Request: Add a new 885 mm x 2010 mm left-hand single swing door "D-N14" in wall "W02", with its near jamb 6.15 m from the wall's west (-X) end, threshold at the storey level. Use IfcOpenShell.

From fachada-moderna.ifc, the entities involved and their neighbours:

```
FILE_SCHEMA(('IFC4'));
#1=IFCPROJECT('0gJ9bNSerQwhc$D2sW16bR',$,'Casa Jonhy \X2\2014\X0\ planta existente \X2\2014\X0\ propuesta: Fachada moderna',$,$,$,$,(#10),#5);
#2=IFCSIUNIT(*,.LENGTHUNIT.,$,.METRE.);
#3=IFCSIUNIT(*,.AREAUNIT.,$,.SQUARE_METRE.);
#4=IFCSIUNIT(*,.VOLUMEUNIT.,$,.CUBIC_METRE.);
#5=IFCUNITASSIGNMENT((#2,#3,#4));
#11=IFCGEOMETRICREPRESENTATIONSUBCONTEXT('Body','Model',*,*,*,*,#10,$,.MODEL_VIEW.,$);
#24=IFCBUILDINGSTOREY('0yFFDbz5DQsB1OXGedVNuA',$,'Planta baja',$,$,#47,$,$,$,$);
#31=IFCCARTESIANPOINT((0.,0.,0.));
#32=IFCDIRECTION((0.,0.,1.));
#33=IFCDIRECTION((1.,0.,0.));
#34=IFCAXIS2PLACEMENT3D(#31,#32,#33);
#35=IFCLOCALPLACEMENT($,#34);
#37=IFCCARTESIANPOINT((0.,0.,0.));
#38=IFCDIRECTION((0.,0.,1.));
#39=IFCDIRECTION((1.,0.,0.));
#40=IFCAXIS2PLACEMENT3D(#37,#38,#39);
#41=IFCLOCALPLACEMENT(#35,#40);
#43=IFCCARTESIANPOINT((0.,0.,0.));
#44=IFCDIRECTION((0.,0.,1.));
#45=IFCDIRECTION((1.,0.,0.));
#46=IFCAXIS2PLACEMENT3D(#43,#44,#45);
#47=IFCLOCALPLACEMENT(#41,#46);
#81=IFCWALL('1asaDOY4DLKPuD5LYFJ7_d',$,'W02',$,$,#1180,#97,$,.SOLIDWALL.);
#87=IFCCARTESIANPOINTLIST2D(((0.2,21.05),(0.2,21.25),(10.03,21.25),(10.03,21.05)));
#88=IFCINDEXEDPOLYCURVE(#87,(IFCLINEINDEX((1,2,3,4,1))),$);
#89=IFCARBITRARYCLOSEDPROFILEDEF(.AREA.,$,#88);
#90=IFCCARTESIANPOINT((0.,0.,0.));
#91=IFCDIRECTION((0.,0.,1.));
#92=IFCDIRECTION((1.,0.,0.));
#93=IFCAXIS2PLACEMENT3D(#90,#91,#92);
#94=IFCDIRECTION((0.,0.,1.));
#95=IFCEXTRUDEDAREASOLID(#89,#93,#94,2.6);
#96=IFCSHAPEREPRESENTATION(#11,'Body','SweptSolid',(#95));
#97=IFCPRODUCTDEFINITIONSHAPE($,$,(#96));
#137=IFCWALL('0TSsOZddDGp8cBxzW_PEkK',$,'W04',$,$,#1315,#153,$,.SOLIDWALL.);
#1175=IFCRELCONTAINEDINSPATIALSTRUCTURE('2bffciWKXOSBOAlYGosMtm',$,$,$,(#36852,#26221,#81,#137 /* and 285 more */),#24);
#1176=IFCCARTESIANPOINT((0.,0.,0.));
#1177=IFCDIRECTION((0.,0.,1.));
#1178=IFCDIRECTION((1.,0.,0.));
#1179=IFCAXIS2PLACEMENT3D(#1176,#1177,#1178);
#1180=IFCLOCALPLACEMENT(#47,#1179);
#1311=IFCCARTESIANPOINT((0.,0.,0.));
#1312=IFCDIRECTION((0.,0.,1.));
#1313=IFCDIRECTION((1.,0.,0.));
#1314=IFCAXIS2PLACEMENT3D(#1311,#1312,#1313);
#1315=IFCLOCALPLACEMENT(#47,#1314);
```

```python
import numpy as np
import ifcopenshell
import ifcopenshell.api.feature
import ifcopenshell.api.geometry
import ifcopenshell.api.root
import ifcopenshell.api.spatial
import ifcopenshell.geom
import ifcopenshell.util.element
import ifcopenshell.util.placement
import ifcopenshell.util.representation
import ifcopenshell.util.shape
import ifcopenshell.util.unit

model = ifcopenshell.open("fachada-moderna.ifc")
unit_scale = ifcopenshell.util.unit.calculate_unit_scale(model)
settings = ifcopenshell.geom.settings()


def volume(element):
    """Net volume in cubic metres, openings subtracted."""
    shape = ifcopenshell.geom.create_shape(settings, element)
    return ifcopenshell.util.shape.get_volume(shape.geometry)


wall = model.by_guid("1asaDOY4DLKPuD5LYFJ7_d")
storey = ifcopenshell.util.element.get_container(wall, ifc_class="IfcBuildingStorey")
context = ifcopenshell.util.representation.get_context(model, "Model", "Body", "MODEL_VIEW")
before = volume(wall)

width, height, from_end, sill = 0.885, 2.01, 6.15, 0.0  # metres

# The wall runs along its own X axis, and the end named is its -X end.
wall_shape = ifcopenshell.geom.create_shape(settings, wall)
x, y, z = ifcopenshell.util.shape.get_vertices(wall_shape.geometry).T
start = x.min() + from_end
face, thickness = float(y.min()), float(y.max() - y.min())
wall_matrix = ifcopenshell.util.placement.get_local_placement(wall.ObjectPlacement)
level = ifcopenshell.util.placement.get_local_placement(storey.ObjectPlacement)[2, 3]


def in_wall(x, y):
    """Placement at x, y metres in the wall's axes, at sill height."""
    matrix = wall_matrix.copy()
    matrix[:, 3] = wall_matrix @ np.array([x / unit_scale, y / unit_scale, 0.0, 1.0])
    matrix[2, 3] = level + sill / unit_scale
    return matrix


# Opening: a box that overshoots both wall faces by 50 mm.
opening = ifcopenshell.api.root.create_entity(model, ifc_class="IfcOpeningElement", predefined_type="OPENING")
box = ifcopenshell.api.geometry.add_wall_representation(
    model, context=context, length=width, height=height, thickness=thickness + 0.1
)
ifcopenshell.api.geometry.assign_representation(model, product=opening, representation=box)
ifcopenshell.api.geometry.edit_object_placement(model, product=opening, matrix=in_wall(start, face - 0.05), is_si=False)
ifcopenshell.api.feature.add_feature(model, feature=opening, element=wall)

door = ifcopenshell.api.root.create_entity(model, ifc_class="IfcDoor", name="D-N14", predefined_type="DOOR")
door.OverallWidth, door.OverallHeight = width / unit_scale, height / unit_scale
door.OperationType = "SINGLE_SWING_LEFT"
body = ifcopenshell.api.geometry.add_door_representation(
    model,
    context=context,
    overall_width=door.OverallWidth,
    overall_height=door.OverallHeight,
    operation_type="SINGLE_SWING_LEFT",
    lining_properties={"LiningDepth": thickness / unit_scale, "ThresholdDepth": thickness / unit_scale},
)
ifcopenshell.api.geometry.assign_representation(model, product=door, representation=body)
ifcopenshell.api.spatial.assign_container(model, products=[door], relating_structure=storey)
ifcopenshell.api.feature.add_filling(model, opening=opening, element=door)

# The lining spans the wall, so the door starts at the wall face.
ifcopenshell.api.geometry.edit_object_placement(model, product=door, matrix=in_wall(start, face), is_si=False)

after = volume(wall)

print(f"wall volume {before:.3f} -> {after:.3f} m3")

model.write("fachada-moderna-out.ifc")
```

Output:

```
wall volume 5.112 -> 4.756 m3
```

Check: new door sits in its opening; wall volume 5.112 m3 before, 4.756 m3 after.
